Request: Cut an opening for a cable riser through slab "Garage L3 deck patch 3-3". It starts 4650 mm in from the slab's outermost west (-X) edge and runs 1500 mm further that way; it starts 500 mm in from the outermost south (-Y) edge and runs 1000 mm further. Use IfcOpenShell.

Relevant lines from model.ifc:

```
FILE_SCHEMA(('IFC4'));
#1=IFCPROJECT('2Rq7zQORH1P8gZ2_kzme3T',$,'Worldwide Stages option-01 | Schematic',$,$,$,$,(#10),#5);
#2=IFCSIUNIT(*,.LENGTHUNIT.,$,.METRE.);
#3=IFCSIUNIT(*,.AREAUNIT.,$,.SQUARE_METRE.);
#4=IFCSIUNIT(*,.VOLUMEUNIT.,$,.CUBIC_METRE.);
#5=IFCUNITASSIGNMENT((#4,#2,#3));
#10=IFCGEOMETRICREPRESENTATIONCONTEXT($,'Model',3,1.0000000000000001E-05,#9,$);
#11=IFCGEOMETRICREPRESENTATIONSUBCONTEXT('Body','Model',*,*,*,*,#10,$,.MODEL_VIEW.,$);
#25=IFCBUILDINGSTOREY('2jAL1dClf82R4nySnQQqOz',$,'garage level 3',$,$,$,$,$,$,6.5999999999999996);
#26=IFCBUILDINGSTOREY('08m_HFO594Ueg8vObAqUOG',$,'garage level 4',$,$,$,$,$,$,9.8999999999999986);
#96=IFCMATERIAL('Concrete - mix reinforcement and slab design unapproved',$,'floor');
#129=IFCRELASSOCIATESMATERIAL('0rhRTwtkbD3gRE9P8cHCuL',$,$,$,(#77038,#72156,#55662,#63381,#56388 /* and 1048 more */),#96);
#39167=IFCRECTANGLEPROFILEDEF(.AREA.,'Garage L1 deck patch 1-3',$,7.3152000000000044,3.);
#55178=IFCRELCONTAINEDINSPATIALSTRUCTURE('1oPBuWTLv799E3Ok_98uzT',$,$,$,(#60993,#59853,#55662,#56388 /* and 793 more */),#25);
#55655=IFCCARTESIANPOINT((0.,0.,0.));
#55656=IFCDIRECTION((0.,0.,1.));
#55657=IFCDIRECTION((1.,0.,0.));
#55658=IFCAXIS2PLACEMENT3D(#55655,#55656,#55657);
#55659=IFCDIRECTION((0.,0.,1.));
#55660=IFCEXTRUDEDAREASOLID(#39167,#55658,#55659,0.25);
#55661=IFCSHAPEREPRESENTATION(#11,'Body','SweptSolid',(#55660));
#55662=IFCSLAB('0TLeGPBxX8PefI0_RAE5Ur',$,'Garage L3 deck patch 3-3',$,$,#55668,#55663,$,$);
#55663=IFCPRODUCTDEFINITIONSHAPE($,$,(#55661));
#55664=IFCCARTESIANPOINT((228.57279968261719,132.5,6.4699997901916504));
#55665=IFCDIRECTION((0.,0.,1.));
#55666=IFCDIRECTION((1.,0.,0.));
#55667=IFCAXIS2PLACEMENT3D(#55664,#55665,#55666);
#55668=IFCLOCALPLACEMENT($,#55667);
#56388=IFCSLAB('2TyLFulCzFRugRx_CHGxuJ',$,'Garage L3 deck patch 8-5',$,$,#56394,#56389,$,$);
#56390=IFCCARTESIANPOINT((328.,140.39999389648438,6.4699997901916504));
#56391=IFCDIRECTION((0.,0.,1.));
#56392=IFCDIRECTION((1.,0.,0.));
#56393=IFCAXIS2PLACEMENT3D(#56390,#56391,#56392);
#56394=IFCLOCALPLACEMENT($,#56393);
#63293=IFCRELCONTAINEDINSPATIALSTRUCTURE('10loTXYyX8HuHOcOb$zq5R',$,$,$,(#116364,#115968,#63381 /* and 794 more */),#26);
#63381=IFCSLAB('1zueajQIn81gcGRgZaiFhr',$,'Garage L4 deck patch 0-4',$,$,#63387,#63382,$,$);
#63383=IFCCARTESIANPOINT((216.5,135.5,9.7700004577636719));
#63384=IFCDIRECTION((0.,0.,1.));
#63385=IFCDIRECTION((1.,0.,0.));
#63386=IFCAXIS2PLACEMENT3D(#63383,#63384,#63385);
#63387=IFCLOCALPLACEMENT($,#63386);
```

```python
import numpy as np
import ifcopenshell
import ifcopenshell.api.feature
import ifcopenshell.api.geometry
import ifcopenshell.api.root
import ifcopenshell.geom
import ifcopenshell.util.placement
import ifcopenshell.util.representation
import ifcopenshell.util.shape
import ifcopenshell.util.unit

model = ifcopenshell.open("model.ifc")
unit_scale = ifcopenshell.util.unit.calculate_unit_scale(model)
settings = ifcopenshell.geom.settings()


def volume(element):
    """Net volume in cubic metres, openings subtracted."""
    shape = ifcopenshell.geom.create_shape(settings, element)
    return ifcopenshell.util.shape.get_volume(shape.geometry)


slab = model.by_guid("0TLeGPBxX8PefI0_RAE5Ur")
before = volume(slab)

# Extent in the slab's own axes, in metres. The edges named are its -X and -Y sides.
slab_shape = ifcopenshell.geom.create_shape(settings, slab)
vertices = ifcopenshell.util.shape.get_vertices(slab_shape.geometry)
x_min, y_min, bottom = vertices.min(axis=0)
top = vertices[:, 2].max()

opening = ifcopenshell.api.root.create_entity(model, ifc_class="IfcOpeningElement", name="Cable riser opening", predefined_type="OPENING")
context = ifcopenshell.util.representation.get_context(model, "Model", "Body", "MODEL_VIEW")
width, depth = 1.5, 1
outline = [(0.0, 0.0), (width, 0.0), (width, depth), (0.0, depth), (0.0, 0.0)]
# Overshoot both faces by 50 mm so the cut is clean.
shape = ifcopenshell.api.geometry.add_slab_representation(
    model, context=context, depth=top - bottom + 0.1, polyline=outline
)
ifcopenshell.api.geometry.assign_representation(model, product=opening, representation=shape)

matrix = ifcopenshell.util.placement.get_local_placement(slab.ObjectPlacement)
matrix[:, 3] = matrix @ np.append(np.array([x_min + 4.65, y_min + 0.5, bottom - 0.05]) / unit_scale, 1.0)
ifcopenshell.api.geometry.edit_object_placement(model, product=opening, matrix=matrix, is_si=False)
ifcopenshell.api.feature.add_feature(model, feature=opening, element=slab)

after = volume(slab)

print(f"slab volume {before:.3f} -> {after:.3f} m3")

model.write("model_rev.ifc")
```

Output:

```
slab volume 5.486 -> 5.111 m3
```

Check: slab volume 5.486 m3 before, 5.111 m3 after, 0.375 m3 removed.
